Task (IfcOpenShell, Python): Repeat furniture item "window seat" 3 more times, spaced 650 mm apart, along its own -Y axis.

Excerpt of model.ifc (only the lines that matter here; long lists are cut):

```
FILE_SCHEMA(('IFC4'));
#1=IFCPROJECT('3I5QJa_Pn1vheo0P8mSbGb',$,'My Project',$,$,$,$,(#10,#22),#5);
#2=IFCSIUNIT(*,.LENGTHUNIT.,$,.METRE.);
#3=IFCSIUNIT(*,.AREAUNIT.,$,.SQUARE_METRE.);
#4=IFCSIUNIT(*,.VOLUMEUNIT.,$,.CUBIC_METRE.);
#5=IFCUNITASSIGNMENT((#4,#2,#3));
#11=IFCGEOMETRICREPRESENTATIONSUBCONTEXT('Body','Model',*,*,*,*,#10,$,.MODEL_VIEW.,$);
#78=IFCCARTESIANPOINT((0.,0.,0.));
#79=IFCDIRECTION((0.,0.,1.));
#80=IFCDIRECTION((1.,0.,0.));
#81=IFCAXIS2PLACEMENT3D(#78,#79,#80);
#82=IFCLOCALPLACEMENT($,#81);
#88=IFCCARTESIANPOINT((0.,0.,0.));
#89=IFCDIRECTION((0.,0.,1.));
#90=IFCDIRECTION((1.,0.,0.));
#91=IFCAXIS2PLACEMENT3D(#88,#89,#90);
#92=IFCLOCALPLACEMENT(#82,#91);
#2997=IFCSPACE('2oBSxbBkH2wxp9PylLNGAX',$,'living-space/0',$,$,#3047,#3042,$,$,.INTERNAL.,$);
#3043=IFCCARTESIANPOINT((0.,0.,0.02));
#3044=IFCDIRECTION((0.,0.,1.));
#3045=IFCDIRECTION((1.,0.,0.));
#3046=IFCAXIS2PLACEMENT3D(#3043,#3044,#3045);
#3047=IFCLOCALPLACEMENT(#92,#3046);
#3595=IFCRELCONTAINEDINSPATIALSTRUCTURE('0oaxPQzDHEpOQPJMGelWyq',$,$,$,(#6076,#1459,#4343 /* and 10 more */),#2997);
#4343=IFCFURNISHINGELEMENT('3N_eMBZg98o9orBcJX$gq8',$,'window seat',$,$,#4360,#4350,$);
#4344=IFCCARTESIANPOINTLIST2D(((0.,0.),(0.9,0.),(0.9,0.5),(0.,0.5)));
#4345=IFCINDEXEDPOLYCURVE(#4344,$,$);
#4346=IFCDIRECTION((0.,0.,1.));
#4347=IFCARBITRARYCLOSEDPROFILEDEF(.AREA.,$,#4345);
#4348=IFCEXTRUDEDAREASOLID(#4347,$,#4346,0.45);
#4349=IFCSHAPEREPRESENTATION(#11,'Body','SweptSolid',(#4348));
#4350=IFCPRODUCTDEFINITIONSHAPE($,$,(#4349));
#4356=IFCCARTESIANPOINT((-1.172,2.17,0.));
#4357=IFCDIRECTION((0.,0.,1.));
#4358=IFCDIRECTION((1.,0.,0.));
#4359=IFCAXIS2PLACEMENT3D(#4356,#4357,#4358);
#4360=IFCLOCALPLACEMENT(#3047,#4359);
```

```python
import ifcopenshell
import ifcopenshell.api.geometry
import ifcopenshell.api.root
import ifcopenshell.util.element
import ifcopenshell.util.placement

model = ifcopenshell.open("model.ifc")

source = model.by_guid("3N_eMBZg98o9orBcJX$gq8")
base = ifcopenshell.util.placement.get_local_placement(source.ObjectPlacement)
step = -base[:3, 1] * 0.65

for i in range(1, 4):
    copy = ifcopenshell.api.root.copy_class(model, product=source)
    copy.Representation = ifcopenshell.util.element.copy_deep(
        model, source.Representation, exclude=["IfcGeometricRepresentationContext", "IfcRepresentationMap"]
    )
    matrix = base.copy()
    matrix[:3, 3] += i * step
    print("added at", matrix[:3, 3].round(3) + 0.0)
    ifcopenshell.api.geometry.edit_object_placement(model, product=copy, matrix=matrix, is_si=False)

model.write("model_rev.ifc")
```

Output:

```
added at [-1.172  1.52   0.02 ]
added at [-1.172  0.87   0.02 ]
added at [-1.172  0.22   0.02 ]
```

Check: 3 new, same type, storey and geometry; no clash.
